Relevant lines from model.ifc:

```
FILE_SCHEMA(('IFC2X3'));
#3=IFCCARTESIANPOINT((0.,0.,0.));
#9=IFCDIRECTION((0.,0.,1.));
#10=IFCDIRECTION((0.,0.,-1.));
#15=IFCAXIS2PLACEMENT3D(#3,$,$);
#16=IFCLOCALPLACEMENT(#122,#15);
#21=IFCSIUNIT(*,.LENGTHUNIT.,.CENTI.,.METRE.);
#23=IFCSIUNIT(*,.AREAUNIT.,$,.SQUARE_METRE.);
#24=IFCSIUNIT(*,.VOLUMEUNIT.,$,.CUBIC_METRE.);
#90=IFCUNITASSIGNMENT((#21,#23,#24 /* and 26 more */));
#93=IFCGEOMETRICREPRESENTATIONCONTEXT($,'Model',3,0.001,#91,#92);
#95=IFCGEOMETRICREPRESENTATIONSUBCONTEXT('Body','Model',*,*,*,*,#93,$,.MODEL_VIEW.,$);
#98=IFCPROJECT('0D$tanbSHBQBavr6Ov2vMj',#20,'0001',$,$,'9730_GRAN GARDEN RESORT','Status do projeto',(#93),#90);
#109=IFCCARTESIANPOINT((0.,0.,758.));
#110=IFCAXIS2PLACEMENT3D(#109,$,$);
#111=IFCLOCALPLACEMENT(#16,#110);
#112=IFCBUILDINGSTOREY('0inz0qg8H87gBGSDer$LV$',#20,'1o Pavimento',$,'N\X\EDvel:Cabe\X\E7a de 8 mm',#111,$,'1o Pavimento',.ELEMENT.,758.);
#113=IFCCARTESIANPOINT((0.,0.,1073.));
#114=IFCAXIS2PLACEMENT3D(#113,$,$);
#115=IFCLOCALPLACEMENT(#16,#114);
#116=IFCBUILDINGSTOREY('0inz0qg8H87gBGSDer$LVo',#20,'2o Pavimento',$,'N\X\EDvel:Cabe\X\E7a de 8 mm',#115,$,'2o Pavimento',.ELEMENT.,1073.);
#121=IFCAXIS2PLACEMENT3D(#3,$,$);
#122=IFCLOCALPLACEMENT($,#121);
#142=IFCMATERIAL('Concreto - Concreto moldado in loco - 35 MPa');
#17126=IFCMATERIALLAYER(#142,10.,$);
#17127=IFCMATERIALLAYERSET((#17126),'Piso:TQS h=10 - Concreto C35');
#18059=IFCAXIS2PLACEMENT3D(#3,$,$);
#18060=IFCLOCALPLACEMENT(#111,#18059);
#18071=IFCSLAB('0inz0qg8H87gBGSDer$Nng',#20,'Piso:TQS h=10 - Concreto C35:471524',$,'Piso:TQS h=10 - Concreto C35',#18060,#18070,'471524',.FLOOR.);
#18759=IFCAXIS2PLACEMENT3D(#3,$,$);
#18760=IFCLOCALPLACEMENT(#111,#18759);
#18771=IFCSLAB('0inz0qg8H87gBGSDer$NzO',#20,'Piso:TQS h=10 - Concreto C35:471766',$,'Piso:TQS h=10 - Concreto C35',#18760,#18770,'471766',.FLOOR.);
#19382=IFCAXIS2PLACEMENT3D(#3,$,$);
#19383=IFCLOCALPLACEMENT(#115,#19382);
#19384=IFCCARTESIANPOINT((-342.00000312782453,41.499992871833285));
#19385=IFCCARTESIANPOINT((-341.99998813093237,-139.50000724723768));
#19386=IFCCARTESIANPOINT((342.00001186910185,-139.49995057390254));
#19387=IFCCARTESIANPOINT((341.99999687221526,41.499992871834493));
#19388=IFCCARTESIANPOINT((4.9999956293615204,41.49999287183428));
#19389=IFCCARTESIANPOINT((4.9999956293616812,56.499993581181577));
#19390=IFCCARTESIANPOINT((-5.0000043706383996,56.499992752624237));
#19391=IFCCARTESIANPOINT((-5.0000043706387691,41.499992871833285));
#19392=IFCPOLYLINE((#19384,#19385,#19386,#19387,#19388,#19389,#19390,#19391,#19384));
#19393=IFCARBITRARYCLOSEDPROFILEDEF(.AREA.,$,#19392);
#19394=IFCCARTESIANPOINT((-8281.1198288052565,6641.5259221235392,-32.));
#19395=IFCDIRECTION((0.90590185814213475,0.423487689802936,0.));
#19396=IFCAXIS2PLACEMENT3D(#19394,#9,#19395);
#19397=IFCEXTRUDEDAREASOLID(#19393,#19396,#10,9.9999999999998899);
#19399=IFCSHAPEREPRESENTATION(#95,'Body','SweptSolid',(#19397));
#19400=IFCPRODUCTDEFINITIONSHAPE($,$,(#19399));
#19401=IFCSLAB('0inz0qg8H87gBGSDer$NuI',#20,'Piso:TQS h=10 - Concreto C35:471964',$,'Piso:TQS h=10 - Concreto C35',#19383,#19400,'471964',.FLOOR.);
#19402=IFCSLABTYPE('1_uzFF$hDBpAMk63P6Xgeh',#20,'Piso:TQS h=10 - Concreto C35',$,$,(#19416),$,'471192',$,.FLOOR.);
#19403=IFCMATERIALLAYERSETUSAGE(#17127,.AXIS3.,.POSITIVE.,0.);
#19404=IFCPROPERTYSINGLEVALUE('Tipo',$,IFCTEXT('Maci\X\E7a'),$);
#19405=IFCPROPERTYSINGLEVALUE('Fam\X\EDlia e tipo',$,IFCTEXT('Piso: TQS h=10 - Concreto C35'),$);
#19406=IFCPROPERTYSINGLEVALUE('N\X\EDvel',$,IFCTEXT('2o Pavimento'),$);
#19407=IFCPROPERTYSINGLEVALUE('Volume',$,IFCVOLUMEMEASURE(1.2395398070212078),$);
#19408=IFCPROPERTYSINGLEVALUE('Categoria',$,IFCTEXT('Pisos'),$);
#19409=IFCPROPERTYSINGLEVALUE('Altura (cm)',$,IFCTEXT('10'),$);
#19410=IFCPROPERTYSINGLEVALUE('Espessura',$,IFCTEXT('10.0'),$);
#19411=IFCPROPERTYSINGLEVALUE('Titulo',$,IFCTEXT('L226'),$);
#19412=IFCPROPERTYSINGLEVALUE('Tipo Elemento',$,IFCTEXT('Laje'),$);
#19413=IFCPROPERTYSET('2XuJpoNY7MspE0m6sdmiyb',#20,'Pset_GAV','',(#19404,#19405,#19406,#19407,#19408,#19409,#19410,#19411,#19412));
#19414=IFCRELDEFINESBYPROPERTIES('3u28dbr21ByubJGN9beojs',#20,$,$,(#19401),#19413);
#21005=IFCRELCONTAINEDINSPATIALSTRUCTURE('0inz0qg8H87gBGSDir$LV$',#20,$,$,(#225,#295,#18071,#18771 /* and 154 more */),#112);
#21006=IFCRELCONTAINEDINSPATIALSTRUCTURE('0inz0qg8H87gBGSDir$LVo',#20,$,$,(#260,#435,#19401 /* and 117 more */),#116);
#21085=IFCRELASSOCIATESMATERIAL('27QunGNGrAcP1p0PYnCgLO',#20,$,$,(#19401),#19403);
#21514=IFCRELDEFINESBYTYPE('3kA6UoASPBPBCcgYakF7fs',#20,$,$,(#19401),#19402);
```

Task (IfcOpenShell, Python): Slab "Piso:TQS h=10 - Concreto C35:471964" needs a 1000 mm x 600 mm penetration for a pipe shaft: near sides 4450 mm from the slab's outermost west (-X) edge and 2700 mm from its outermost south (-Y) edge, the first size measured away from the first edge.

```python
import numpy as np
import ifcopenshell
import ifcopenshell.api.feature
import ifcopenshell.api.geometry
import ifcopenshell.api.pset
import ifcopenshell.api.root
import ifcopenshell.geom
import ifcopenshell.util.element
import ifcopenshell.util.placement
import ifcopenshell.util.representation
import ifcopenshell.util.shape
import ifcopenshell.util.unit

model = ifcopenshell.open("model.ifc")
unit_scale = ifcopenshell.util.unit.calculate_unit_scale(model)
volume_scale = ifcopenshell.util.unit.calculate_unit_scale(model, "VOLUMEUNIT")
settings = ifcopenshell.geom.settings()


def volume(element):
    """Net volume in cubic metres, openings subtracted."""
    shape = ifcopenshell.geom.create_shape(settings, element)
    return ifcopenshell.util.shape.get_volume(shape.geometry)


slab = model.by_guid("0inz0qg8H87gBGSDer$NuI")
before = volume(slab)

# Extent in the slab's own axes, in metres. The edges named are its -X and -Y sides.
slab_shape = ifcopenshell.geom.create_shape(settings, slab)
vertices = ifcopenshell.util.shape.get_vertices(slab_shape.geometry)
x_min, y_min, bottom = vertices.min(axis=0)
top = vertices[:, 2].max()

opening = ifcopenshell.api.root.create_entity(model, ifc_class="IfcOpeningElement", name="Pipe shaft opening")
context = ifcopenshell.util.representation.get_context(model, "Model", "Body", "MODEL_VIEW")
width, depth = 1, 0.6
outline = [(0.0, 0.0), (width, 0.0), (width, depth), (0.0, depth), (0.0, 0.0)]
# Overshoot both faces by 50 mm so the cut is clean.
shape = ifcopenshell.api.geometry.add_slab_representation(
    model, context=context, depth=top - bottom + 0.1, polyline=outline
)
ifcopenshell.api.geometry.assign_representation(model, product=opening, representation=shape)

matrix = ifcopenshell.util.placement.get_local_placement(slab.ObjectPlacement)
matrix[:, 3] = matrix @ np.append(np.array([x_min + 4.45, y_min + 2.7, bottom - 0.05]) / unit_scale, 1.0)
ifcopenshell.api.geometry.edit_object_placement(model, product=opening, matrix=matrix, is_si=False)
ifcopenshell.api.feature.add_feature(model, feature=opening, element=slab)

after = volume(slab)

# Update the slab's stored quantities.
pset = model.by_id(ifcopenshell.util.element.get_pset(slab, "Pset_GAV", should_inherit=False)["id"])
ifcopenshell.api.pset.edit_pset(model, pset=pset, properties={
    "Volume": model.create_entity("IfcVolumeMeasure", after / volume_scale),
})

print(f"slab volume {before:.3f} -> {after:.3f} m3")

model.write("model_v2.ifc")
```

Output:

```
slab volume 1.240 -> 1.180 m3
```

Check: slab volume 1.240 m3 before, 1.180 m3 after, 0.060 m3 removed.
